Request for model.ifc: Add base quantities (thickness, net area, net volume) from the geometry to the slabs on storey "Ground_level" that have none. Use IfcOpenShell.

First a look at what the model holds.

```python
import ifcopenshell
import ifcopenshell.util.element
import ifcopenshell.util.unit

model = ifcopenshell.open("model.ifc")
print(model.schema)
for unit_type in ("LENGTHUNIT", "AREAUNIT", "VOLUMEUNIT"):
    print(unit_type, ifcopenshell.util.unit.calculate_unit_scale(model, unit_type))
storey = next(s for s in model.by_type("IfcBuildingStorey") if s.Name == "Ground_level")
slabs = [e for e in ifcopenshell.util.element.get_decomposition(storey) if e.is_a("IfcSlab")]
for e in sorted(slabs, key=lambda e: e.id()):
    print(e.id(), e.is_a(), e.Name, list(ifcopenshell.util.element.get_psets(e, qtos_only=True)), sep=" | ")
```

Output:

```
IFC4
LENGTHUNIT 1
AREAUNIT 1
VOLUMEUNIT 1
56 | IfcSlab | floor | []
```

```python
import ifcopenshell
import ifcopenshell.api.pset
import ifcopenshell.geom
import ifcopenshell.util.element
import ifcopenshell.util.shape
import ifcopenshell.util.unit

model = ifcopenshell.open("model.ifc")
unit_scale = ifcopenshell.util.unit.calculate_unit_scale(model)
area_scale = ifcopenshell.util.unit.calculate_unit_scale(model, "AREAUNIT")
volume_scale = ifcopenshell.util.unit.calculate_unit_scale(model, "VOLUMEUNIT")
settings = ifcopenshell.geom.settings()

storey = next(s for s in model.by_type("IfcBuildingStorey") if s.Name == "Ground_level")
slabs = [e for e in ifcopenshell.util.element.get_decomposition(storey) if e.is_a("IfcSlab")]

for e in sorted(slabs, key=lambda e: e.id()):
    if ifcopenshell.util.element.get_psets(e, qtos_only=True, should_inherit=False):
        continue
    # Geometry comes back in metres, in the element's own axes.
    shape = ifcopenshell.geom.create_shape(settings, e)
    values = {
        "Width": ifcopenshell.util.shape.get_z(shape.geometry) / unit_scale,
        "NetArea": ifcopenshell.util.shape.get_footprint_area(shape.geometry) / area_scale,
        "NetVolume": ifcopenshell.util.shape.get_volume(shape.geometry) / volume_scale,
    }
    qto = ifcopenshell.api.pset.add_qto(model, product=e, name="Qto_SlabBaseQuantities")
    ifcopenshell.api.pset.edit_qto(model, qto=qto, properties=values)
    print(e.id(), {k: round(v, 3) for k, v in values.items()})

model.write("model_updated.ifc")
```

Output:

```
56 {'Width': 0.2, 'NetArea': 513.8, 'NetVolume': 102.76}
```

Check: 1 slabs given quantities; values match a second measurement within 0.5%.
